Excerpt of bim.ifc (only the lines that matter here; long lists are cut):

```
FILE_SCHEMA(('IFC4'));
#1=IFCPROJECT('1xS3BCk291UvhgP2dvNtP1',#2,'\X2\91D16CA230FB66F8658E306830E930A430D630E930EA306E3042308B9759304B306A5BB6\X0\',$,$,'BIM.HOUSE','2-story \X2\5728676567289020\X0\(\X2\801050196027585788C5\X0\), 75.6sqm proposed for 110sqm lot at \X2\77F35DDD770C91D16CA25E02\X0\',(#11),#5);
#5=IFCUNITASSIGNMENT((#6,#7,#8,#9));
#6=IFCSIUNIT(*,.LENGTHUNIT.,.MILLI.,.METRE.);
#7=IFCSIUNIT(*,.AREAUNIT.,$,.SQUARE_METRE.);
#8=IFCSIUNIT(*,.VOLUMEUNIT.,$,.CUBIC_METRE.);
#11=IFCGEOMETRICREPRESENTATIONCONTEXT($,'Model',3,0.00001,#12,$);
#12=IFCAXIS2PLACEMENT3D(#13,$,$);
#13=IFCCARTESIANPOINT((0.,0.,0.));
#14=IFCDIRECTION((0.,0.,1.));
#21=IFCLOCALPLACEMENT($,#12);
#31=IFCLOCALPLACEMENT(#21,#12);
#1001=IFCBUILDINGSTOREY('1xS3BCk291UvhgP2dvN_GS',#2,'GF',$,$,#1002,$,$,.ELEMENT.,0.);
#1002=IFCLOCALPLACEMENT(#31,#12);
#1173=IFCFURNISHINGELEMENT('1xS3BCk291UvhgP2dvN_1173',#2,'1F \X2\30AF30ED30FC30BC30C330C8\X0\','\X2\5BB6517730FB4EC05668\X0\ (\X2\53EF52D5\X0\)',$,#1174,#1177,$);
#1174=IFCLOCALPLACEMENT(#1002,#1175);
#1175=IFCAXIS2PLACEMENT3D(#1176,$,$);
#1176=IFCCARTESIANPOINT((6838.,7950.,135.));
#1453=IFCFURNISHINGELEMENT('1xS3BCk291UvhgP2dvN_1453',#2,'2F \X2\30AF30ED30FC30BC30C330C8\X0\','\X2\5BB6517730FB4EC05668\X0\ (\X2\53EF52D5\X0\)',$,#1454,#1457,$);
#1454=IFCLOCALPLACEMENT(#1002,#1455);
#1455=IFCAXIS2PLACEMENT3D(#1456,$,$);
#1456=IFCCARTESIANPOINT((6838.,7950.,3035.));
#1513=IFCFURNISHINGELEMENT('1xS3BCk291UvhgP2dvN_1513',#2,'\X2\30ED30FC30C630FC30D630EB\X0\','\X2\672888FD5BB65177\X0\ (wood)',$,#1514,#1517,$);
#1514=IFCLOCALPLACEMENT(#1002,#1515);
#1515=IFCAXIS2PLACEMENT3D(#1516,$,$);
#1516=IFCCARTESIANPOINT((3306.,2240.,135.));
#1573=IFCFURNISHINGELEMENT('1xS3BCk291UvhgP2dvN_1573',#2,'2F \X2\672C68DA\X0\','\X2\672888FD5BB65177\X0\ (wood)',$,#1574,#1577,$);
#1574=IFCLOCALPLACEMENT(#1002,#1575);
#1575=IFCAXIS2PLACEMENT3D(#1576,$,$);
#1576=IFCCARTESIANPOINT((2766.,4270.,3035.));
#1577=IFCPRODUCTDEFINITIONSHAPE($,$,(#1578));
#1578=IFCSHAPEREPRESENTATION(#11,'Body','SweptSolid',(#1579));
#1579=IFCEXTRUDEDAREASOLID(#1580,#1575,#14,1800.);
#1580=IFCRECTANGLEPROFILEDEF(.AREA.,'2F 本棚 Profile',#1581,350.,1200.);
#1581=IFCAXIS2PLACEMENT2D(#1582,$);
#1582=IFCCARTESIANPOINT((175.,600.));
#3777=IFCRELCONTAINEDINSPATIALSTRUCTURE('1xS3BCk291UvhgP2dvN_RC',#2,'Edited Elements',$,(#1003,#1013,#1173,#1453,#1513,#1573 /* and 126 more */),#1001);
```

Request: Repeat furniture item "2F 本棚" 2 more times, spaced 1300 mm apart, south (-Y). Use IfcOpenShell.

```python
import numpy as np
import ifcopenshell
import ifcopenshell.api.geometry
import ifcopenshell.api.root
import ifcopenshell.util.element
import ifcopenshell.util.placement
import ifcopenshell.util.unit

model = ifcopenshell.open("bim.ifc")
unit_scale = ifcopenshell.util.unit.calculate_unit_scale(model)


def reuse_history(source, copy):
    """copy_class also copies each property set's owner history, people and application; keep the originals."""
    for rel in copy.IsDefinedBy:
        if rel.is_a("IfcRelDefinesByProperties") and (history := rel.RelatingPropertyDefinition.OwnerHistory):
            rel.RelatingPropertyDefinition.OwnerHistory = source.OwnerHistory
            ifcopenshell.util.element.remove_deep2(model, history)


source = model.by_guid("1xS3BCk291UvhgP2dvN_1573")
base = ifcopenshell.util.placement.get_local_placement(source.ObjectPlacement)
step = np.array([0.0, -1.0, 0.0]) * 1.3 / unit_scale

for i in range(1, 3):
    copy = ifcopenshell.api.root.copy_class(model, product=source)
    copy.Representation = ifcopenshell.util.element.copy_deep(
        model, source.Representation, exclude=["IfcGeometricRepresentationContext", "IfcRepresentationMap"]
    )
    reuse_history(source, copy)
    matrix = base.copy()
    matrix[:3, 3] += i * step
    print("added at", matrix[:3, 3].round(3) + 0.0)
    ifcopenshell.api.geometry.edit_object_placement(model, product=copy, matrix=matrix, is_si=False)

model.write("bim_updated.ifc")
```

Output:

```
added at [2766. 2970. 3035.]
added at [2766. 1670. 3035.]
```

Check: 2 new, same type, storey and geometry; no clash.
